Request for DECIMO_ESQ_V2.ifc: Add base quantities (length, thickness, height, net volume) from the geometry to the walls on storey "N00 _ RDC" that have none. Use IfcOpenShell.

First a look at what the model holds.

```python
import ifcopenshell
import ifcopenshell.util.element
import ifcopenshell.util.unit

model = ifcopenshell.open("DECIMO_ESQ_V2.ifc")
print(model.schema)
for unit_type in ("LENGTHUNIT", "AREAUNIT", "VOLUMEUNIT"):
    print(unit_type, ifcopenshell.util.unit.calculate_unit_scale(model, unit_type))
storey = next(s for s in model.by_type("IfcBuildingStorey") if s.Name == "N00 _ RDC")
walls = [e for e in ifcopenshell.util.element.get_decomposition(storey) if e.is_a("IfcWall")]
for e in sorted(walls, key=lambda e: e.id()):
    print(e.id(), e.is_a(), e.Name, list(ifcopenshell.util.element.get_psets(e, qtos_only=True)), sep=" | ")
```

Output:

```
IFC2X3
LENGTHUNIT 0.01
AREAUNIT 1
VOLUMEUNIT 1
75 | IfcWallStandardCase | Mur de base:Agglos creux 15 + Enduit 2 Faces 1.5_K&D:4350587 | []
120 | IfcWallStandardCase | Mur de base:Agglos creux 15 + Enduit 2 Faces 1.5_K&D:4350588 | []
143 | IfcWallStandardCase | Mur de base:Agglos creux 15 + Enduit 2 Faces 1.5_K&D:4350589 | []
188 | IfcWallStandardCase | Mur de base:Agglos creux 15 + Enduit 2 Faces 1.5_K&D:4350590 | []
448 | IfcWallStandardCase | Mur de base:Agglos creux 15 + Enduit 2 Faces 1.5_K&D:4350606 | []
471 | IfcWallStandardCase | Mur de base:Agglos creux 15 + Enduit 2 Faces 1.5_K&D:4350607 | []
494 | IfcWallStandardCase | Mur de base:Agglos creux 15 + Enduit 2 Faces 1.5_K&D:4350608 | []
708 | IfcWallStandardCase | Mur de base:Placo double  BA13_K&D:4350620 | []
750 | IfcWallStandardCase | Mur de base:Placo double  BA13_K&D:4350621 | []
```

```python
import ifcopenshell
import ifcopenshell.api.pset
import ifcopenshell.geom
import ifcopenshell.util.element
import ifcopenshell.util.shape
import ifcopenshell.util.unit

model = ifcopenshell.open("DECIMO_ESQ_V2.ifc")
unit_scale = ifcopenshell.util.unit.calculate_unit_scale(model)
volume_scale = ifcopenshell.util.unit.calculate_unit_scale(model, "VOLUMEUNIT")
settings = ifcopenshell.geom.settings()

storey = next(s for s in model.by_type("IfcBuildingStorey") if s.Name == "N00 _ RDC")
walls = [e for e in ifcopenshell.util.element.get_decomposition(storey) if e.is_a("IfcWall")]

for e in sorted(walls, key=lambda e: e.id()):
    if ifcopenshell.util.element.get_psets(e, qtos_only=True, should_inherit=False):
        continue
    # Geometry comes back in metres, in the element's own axes.
    shape = ifcopenshell.geom.create_shape(settings, e)
    values = {
        "Length": ifcopenshell.util.shape.get_x(shape.geometry) / unit_scale,
        "Width": ifcopenshell.util.shape.get_y(shape.geometry) / unit_scale,
        "Height": ifcopenshell.util.shape.get_z(shape.geometry) / unit_scale,
        "NetVolume": ifcopenshell.util.shape.get_volume(shape.geometry) / volume_scale,
    }
    qto = ifcopenshell.api.pset.add_qto(model, product=e, name="BaseQuantities")
    ifcopenshell.api.pset.edit_qto(model, qto=qto, properties=values)
    print(e.id(), {k: round(v, 3) for k, v in values.items()})

model.write("DECIMO_ESQ_V2_v2.ifc")
```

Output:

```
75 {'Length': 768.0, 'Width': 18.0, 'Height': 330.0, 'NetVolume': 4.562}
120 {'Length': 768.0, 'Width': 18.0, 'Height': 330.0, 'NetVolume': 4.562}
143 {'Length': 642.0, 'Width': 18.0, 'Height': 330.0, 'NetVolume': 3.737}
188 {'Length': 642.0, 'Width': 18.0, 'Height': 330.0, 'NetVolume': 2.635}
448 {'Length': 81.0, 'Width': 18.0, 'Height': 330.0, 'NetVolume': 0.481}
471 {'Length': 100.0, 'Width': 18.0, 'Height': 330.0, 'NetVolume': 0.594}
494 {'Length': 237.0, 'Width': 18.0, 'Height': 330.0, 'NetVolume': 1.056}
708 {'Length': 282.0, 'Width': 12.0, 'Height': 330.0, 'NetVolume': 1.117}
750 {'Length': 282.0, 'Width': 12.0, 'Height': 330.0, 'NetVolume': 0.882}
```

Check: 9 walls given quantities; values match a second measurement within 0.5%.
